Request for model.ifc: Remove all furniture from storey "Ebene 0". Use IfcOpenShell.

First a look at what the model holds.

```python
import ifcopenshell
import ifcopenshell.util.element

model = ifcopenshell.open("model.ifc")
print(model.schema)
storey = next(s for s in model.by_type("IfcBuildingStorey") if s.Name == "Ebene 0")
furniture = [e for e in ifcopenshell.util.element.get_decomposition(storey) if e.is_a("IfcFurnishingElement")]
seen = {}
for e in furniture:
    element_type = ifcopenshell.util.element.get_type(e)
    name = element_type.Name if element_type not in (None, e) else None
    seen[name] = seen.get(name, 0) + 1
for name, count in sorted(seen.items(), key=str):
    print(count, "x", name)
```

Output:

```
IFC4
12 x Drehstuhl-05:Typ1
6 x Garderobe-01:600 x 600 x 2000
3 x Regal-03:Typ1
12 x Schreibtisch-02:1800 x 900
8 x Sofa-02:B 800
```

```python
import ifcopenshell
import ifcopenshell.api.root
import ifcopenshell.util.element

model = ifcopenshell.open("model.ifc")

storey = next(s for s in model.by_type("IfcBuildingStorey") if s.Name == "Ebene 0")
furniture = [e for e in ifcopenshell.util.element.get_decomposition(storey) if e.is_a("IfcFurnishingElement")]

for e in furniture:
    ifcopenshell.api.root.remove_product(model, product=e)
print(len(furniture), "removed")

model.write("model_v2.ifc")
```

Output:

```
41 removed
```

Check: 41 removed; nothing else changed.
